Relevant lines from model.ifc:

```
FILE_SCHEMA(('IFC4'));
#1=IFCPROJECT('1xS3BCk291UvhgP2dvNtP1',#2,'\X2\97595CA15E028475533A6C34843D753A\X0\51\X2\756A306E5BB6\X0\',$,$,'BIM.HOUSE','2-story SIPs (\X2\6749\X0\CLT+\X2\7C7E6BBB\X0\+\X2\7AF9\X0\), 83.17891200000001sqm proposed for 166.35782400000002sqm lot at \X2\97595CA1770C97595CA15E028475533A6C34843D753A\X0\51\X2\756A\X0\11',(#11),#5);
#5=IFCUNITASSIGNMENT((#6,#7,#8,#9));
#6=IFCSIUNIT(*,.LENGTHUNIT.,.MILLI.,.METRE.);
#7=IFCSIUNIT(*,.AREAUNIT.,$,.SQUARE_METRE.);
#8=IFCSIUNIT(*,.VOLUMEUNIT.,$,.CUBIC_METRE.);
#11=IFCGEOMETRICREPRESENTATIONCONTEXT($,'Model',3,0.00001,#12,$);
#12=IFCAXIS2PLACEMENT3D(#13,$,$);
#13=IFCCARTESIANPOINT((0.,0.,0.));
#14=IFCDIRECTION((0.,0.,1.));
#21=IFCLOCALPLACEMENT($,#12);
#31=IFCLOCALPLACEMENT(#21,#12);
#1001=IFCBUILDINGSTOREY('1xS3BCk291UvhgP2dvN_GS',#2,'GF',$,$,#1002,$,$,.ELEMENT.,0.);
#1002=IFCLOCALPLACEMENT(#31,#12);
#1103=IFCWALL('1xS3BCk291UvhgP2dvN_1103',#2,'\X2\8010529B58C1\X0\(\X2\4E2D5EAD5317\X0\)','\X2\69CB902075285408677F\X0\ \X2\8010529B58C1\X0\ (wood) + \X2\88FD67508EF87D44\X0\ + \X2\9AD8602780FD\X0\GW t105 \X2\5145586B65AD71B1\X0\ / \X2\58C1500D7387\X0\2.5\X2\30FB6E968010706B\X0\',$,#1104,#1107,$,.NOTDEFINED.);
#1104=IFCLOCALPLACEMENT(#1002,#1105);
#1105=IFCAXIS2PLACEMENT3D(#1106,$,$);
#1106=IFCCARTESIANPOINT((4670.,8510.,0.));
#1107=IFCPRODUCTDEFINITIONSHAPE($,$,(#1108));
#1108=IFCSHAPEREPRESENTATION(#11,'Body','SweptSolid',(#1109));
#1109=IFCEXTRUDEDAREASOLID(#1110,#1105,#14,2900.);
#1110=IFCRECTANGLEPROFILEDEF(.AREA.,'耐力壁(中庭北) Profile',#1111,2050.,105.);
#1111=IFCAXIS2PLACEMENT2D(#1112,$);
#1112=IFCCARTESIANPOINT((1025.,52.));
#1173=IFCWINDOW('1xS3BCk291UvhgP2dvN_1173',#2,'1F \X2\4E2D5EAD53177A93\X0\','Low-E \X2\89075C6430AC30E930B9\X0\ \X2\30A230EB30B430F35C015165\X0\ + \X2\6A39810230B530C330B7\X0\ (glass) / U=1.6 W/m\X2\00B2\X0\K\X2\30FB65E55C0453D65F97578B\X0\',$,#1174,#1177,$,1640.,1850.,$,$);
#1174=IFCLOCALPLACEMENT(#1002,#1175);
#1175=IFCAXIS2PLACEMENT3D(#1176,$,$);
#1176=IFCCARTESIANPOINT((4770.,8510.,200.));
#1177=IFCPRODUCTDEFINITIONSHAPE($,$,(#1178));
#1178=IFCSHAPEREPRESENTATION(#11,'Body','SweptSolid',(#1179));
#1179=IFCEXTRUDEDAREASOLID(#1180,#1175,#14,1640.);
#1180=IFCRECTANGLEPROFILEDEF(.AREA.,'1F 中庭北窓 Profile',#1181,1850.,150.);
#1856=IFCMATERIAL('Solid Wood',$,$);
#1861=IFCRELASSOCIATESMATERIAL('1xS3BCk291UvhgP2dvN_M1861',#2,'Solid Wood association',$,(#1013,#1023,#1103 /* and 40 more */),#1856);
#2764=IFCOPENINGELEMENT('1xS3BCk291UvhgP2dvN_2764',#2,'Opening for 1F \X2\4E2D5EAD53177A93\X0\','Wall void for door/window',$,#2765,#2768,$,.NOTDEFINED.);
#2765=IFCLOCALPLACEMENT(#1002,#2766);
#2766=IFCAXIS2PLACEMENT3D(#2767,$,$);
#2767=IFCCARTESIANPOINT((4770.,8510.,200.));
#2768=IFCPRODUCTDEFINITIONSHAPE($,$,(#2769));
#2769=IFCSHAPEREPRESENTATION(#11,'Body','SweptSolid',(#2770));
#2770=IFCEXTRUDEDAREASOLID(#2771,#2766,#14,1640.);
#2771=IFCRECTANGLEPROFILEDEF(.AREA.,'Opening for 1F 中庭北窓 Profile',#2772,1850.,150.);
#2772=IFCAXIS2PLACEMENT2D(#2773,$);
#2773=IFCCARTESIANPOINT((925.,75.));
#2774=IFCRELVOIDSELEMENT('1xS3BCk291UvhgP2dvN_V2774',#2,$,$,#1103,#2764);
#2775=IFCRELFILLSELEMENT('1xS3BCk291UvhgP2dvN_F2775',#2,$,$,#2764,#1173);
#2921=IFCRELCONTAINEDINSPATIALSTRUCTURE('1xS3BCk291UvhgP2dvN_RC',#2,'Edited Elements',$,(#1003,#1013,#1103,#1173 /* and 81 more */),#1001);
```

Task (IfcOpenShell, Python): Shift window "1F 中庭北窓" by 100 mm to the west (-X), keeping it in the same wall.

```python
import ifcopenshell
import ifcopenshell.api.geometry
import ifcopenshell.util.placement
import ifcopenshell.util.unit

model = ifcopenshell.open("model.ifc")
unit_scale = ifcopenshell.util.unit.calculate_unit_scale(model)

window = model.by_guid("1xS3BCk291UvhgP2dvN_1173")
opening = window.FillsVoids[0].RelatingOpeningElement
wall = opening.VoidsElements[0].RelatingBuildingElement

wall_matrix = ifcopenshell.util.placement.get_local_placement(wall.ObjectPlacement)
shift = wall_matrix[:3, 0] * -0.1 / unit_scale
before = ifcopenshell.util.placement.get_local_placement(window.ObjectPlacement)[:3, 3].copy()

# The window is not placed relative to its opening, so move both.
for product in (opening, window):
    matrix = ifcopenshell.util.placement.get_local_placement(product.ObjectPlacement)
    matrix[:3, 3] += shift
    ifcopenshell.api.geometry.edit_object_placement(model, product=product, matrix=matrix, is_si=False)

after = ifcopenshell.util.placement.get_local_placement(window.ObjectPlacement)[:3, 3]
print("window moved by", (after - before).round(3) + 0.0)

model.write("model_v2.ifc")
```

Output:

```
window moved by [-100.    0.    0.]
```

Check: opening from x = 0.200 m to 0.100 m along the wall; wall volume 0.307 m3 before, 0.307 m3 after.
